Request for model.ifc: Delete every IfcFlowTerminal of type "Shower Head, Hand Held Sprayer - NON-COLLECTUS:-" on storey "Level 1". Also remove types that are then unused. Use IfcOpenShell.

First a look at what the model holds.

```python
import ifcopenshell
import ifcopenshell.util.element

model = ifcopenshell.open("model.ifc")
print(model.schema)
storey = next(s for s in model.by_type("IfcBuildingStorey") if s.Name == "Level 1")
terminals = [e for e in ifcopenshell.util.element.get_decomposition(storey) if e.is_a("IfcFlowTerminal")]
seen = {}
for e in terminals:
    element_type = ifcopenshell.util.element.get_type(e)
    name = element_type.Name if element_type not in (None, e) else None
    seen[name] = seen.get(name, 0) + 1
for name, count in sorted(seen.items(), key=str):
    print(count, "x", name)
```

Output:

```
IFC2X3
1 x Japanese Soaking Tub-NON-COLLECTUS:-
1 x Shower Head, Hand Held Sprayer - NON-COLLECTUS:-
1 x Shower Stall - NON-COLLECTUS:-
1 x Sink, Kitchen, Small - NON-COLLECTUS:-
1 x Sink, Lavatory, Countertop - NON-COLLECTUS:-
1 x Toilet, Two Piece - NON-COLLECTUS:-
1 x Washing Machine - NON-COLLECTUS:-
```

```python
import ifcopenshell
import ifcopenshell.api.root
import ifcopenshell.util.element

model = ifcopenshell.open("model.ifc")

storey = next(s for s in model.by_type("IfcBuildingStorey") if s.Name == "Level 1")
terminals = [e for e in ifcopenshell.util.element.get_decomposition(storey) if e.is_a("IfcFlowTerminal")]
targets = [e for e in terminals if (t := ifcopenshell.util.element.get_type(e)) not in (None, e) and t.Name == "Shower Head, Hand Held Sprayer - NON-COLLECTUS:-"]
types = {ifcopenshell.util.element.get_type(e) for e in targets} - {None, *targets}

for e in targets:
    ifcopenshell.api.root.remove_product(model, product=e)
print(len(targets), "removed")

unused = [t for t in types if not ifcopenshell.util.element.get_types(t)]
for t in unused:
    ifcopenshell.api.root.remove_product(model, product=t)
print(len(unused), "unused types removed")

model.write("model_rev.ifc")
```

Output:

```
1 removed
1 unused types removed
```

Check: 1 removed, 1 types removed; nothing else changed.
